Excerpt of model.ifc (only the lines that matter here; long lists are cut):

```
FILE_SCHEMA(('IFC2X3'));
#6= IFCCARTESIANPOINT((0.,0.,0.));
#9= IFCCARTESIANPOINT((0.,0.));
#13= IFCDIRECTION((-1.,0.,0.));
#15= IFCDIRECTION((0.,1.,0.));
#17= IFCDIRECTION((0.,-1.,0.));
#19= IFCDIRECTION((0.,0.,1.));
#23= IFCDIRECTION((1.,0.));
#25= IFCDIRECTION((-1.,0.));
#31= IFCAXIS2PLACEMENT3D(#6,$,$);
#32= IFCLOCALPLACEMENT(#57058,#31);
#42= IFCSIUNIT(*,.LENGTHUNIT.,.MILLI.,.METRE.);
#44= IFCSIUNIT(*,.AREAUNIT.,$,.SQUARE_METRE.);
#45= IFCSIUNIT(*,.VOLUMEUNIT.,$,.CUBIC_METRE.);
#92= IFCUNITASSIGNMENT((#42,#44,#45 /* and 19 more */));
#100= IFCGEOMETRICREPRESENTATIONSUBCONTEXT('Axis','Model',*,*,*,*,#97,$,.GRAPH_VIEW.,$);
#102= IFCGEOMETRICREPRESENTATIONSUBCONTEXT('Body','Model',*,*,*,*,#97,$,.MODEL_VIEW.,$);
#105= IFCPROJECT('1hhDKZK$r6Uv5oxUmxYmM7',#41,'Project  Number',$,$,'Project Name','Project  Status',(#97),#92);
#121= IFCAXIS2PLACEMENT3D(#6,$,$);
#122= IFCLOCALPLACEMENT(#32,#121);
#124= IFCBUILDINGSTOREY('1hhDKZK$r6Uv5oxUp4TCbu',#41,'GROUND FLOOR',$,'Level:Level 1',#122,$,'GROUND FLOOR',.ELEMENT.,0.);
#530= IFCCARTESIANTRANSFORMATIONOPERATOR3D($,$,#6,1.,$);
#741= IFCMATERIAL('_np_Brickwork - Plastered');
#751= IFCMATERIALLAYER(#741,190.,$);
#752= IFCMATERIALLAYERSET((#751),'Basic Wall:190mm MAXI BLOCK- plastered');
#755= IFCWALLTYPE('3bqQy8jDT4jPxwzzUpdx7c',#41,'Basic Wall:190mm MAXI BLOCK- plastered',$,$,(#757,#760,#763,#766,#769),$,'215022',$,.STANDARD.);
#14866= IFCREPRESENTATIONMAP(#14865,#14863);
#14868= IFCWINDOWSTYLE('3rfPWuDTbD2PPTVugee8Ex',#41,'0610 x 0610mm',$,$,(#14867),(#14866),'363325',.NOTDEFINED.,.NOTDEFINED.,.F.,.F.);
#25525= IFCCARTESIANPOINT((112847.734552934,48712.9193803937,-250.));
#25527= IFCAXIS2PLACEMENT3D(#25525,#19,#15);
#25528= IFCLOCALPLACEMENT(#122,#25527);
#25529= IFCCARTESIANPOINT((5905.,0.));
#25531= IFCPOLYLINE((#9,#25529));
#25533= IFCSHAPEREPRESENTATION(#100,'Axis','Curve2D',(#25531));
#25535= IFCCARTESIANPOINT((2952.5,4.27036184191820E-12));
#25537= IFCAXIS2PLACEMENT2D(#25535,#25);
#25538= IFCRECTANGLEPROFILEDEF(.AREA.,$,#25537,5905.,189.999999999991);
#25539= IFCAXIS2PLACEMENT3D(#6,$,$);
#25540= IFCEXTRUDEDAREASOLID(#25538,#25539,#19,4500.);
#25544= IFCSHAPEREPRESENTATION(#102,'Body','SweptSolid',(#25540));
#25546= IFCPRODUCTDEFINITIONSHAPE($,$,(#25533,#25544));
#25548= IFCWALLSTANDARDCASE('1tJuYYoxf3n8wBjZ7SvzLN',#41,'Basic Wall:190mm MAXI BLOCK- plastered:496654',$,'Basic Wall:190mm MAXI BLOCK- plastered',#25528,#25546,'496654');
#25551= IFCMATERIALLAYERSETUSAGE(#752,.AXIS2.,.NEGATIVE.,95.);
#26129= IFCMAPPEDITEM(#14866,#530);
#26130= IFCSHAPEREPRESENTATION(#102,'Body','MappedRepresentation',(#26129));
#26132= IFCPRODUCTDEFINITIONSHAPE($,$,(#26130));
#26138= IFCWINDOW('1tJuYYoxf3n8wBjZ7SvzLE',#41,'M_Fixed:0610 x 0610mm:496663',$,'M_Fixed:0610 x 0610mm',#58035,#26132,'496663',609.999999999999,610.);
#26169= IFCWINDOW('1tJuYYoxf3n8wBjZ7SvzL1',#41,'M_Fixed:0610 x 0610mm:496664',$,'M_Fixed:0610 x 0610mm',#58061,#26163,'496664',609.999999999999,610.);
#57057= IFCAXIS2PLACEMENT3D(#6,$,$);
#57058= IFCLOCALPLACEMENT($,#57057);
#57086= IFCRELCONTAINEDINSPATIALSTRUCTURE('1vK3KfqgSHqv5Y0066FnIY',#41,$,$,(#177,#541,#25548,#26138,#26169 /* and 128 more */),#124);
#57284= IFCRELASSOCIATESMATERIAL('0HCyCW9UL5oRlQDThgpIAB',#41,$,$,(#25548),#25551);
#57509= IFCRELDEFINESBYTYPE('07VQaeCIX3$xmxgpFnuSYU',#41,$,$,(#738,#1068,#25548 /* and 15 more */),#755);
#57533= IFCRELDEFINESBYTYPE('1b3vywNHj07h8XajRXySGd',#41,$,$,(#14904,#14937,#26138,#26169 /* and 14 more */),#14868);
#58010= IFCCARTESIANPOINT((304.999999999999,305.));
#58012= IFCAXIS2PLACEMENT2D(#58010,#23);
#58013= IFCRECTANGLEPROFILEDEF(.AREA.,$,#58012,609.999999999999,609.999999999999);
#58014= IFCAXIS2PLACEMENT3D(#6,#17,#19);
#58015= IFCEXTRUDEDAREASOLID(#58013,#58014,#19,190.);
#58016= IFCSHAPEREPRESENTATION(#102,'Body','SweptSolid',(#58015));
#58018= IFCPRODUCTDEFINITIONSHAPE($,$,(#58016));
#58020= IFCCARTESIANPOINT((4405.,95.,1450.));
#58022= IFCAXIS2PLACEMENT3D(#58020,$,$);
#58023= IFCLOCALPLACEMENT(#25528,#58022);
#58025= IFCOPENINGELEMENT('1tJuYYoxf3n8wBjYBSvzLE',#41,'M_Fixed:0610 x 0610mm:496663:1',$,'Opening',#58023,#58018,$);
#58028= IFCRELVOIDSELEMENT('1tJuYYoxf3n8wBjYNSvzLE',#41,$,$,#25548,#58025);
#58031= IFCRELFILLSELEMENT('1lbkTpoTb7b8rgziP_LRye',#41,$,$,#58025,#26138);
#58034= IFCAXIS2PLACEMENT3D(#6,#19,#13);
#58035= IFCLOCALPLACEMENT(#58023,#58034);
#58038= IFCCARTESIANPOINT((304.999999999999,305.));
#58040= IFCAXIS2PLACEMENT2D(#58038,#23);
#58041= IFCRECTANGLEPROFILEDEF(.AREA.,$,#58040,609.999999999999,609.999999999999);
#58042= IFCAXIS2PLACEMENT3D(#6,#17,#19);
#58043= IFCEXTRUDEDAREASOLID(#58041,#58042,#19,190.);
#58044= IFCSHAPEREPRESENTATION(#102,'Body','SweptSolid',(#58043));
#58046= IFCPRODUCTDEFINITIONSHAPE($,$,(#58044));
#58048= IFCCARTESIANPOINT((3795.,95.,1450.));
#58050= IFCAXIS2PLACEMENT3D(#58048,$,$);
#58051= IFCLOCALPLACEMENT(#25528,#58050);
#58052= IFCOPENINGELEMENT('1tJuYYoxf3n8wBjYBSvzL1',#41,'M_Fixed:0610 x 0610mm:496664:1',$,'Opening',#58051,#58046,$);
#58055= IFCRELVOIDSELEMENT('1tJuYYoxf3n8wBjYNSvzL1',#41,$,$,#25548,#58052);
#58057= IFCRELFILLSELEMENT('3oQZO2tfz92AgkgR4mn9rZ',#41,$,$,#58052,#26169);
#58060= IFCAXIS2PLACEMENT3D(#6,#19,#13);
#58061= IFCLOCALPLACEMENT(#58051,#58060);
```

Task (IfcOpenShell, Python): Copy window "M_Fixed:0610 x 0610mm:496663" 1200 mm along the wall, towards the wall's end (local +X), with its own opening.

```python
import ifcopenshell
import ifcopenshell.api.feature
import ifcopenshell.api.geometry
import ifcopenshell.api.root
import ifcopenshell.geom
import ifcopenshell.util.element
import ifcopenshell.util.placement
import ifcopenshell.util.shape

model = ifcopenshell.open("model.ifc")
settings = ifcopenshell.geom.settings()


def volume(element):
    """Net volume in cubic metres, openings subtracted."""
    shape = ifcopenshell.geom.create_shape(settings, element)
    return ifcopenshell.util.shape.get_volume(shape.geometry)


def reuse_history(source, copy):
    """copy_class also copies each property set's owner history, people and application; keep the originals."""
    for rel in copy.IsDefinedBy:
        if rel.is_a("IfcRelDefinesByProperties") and (history := rel.RelatingPropertyDefinition.OwnerHistory):
            rel.RelatingPropertyDefinition.OwnerHistory = source.OwnerHistory
            ifcopenshell.util.element.remove_deep2(model, history)


window = model.by_guid("1tJuYYoxf3n8wBjZ7SvzLE")
opening = window.FillsVoids[0].RelatingOpeningElement
wall = opening.VoidsElements[0].RelatingBuildingElement
before = volume(wall)
shift = ifcopenshell.util.placement.get_local_placement(wall.ObjectPlacement)[:3, 0] * 1200.0

# copy_class copies the void relationship, type, container and properties, but no geometry.
new_opening = ifcopenshell.api.root.copy_class(model, product=opening)
new_opening.Representation = ifcopenshell.util.element.copy_deep(
    model, opening.Representation, exclude=["IfcGeometricRepresentationContext", "IfcRepresentationMap"]
)
new_opening.Name = "M_Fixed:0610 x 0610mm"
new_window = ifcopenshell.api.root.copy_class(model, product=window)
new_window.Representation = ifcopenshell.util.element.copy_deep(
    model, window.Representation, exclude=["IfcGeometricRepresentationContext", "IfcRepresentationMap"]
)
new_window.Name = "M_Fixed:0610 x 0610mm"
new_window.Tag = None
reuse_history(window, new_window)
fills = ifcopenshell.api.feature.add_filling(model, opening=new_opening, element=new_window)
fills.OwnerHistory = new_window.OwnerHistory  # required in IFC2X3

for old, new in ((opening, new_opening), (window, new_window)):
    matrix = ifcopenshell.util.placement.get_local_placement(old.ObjectPlacement)
    matrix[:3, 3] += shift
    ifcopenshell.api.geometry.edit_object_placement(model, product=new, matrix=matrix, is_si=False)

after = volume(wall)

print(f"wall volume {before:.3f} -> {after:.3f} m3")

model.write("model_updated.ifc")
```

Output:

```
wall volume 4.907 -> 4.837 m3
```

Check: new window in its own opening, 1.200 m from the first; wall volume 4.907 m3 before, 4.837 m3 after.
